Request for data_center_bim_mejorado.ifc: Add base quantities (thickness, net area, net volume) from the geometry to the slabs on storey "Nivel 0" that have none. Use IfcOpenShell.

First a look at what the model holds.

```python
import ifcopenshell
import ifcopenshell.util.element
import ifcopenshell.util.unit

model = ifcopenshell.open("data_center_bim_mejorado.ifc")
print(model.schema)
for unit_type in ("LENGTHUNIT", "AREAUNIT", "VOLUMEUNIT"):
    print(unit_type, ifcopenshell.util.unit.calculate_unit_scale(model, unit_type))
storey = next(s for s in model.by_type("IfcBuildingStorey") if s.Name == "Nivel 0")
slabs = [e for e in ifcopenshell.util.element.get_decomposition(storey) if e.is_a("IfcSlab")]
for e in sorted(slabs, key=lambda e: e.id()):
    print(e.id(), e.is_a(), e.Name, list(ifcopenshell.util.element.get_psets(e, qtos_only=True)), sep=" | ")
```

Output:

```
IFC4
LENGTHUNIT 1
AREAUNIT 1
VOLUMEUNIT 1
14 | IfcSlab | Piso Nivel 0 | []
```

```python
import ifcopenshell
import ifcopenshell.api.pset
import ifcopenshell.geom
import ifcopenshell.util.element
import ifcopenshell.util.shape
import ifcopenshell.util.unit

model = ifcopenshell.open("data_center_bim_mejorado.ifc")
unit_scale = ifcopenshell.util.unit.calculate_unit_scale(model)
area_scale = ifcopenshell.util.unit.calculate_unit_scale(model, "AREAUNIT")
volume_scale = ifcopenshell.util.unit.calculate_unit_scale(model, "VOLUMEUNIT")
settings = ifcopenshell.geom.settings()

storey = next(s for s in model.by_type("IfcBuildingStorey") if s.Name == "Nivel 0")
slabs = [e for e in ifcopenshell.util.element.get_decomposition(storey) if e.is_a("IfcSlab")]

for e in sorted(slabs, key=lambda e: e.id()):
    if ifcopenshell.util.element.get_psets(e, qtos_only=True, should_inherit=False):
        continue
    # Geometry comes back in metres, in the element's own axes.
    shape = ifcopenshell.geom.create_shape(settings, e)
    values = {
        "Width": ifcopenshell.util.shape.get_z(shape.geometry) / unit_scale,
        "NetArea": ifcopenshell.util.shape.get_footprint_area(shape.geometry) / area_scale,
        "NetVolume": ifcopenshell.util.shape.get_volume(shape.geometry) / volume_scale,
    }
    qto = ifcopenshell.api.pset.add_qto(model, product=e, name="Qto_SlabBaseQuantities")
    ifcopenshell.api.pset.edit_qto(model, qto=qto, properties=values)
    print(e.id(), {k: round(v, 3) for k, v in values.items()})

model.write("data_center_bim_mejorado_rev.ifc")
```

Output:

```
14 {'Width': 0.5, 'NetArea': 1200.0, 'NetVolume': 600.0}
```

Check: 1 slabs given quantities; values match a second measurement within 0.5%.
